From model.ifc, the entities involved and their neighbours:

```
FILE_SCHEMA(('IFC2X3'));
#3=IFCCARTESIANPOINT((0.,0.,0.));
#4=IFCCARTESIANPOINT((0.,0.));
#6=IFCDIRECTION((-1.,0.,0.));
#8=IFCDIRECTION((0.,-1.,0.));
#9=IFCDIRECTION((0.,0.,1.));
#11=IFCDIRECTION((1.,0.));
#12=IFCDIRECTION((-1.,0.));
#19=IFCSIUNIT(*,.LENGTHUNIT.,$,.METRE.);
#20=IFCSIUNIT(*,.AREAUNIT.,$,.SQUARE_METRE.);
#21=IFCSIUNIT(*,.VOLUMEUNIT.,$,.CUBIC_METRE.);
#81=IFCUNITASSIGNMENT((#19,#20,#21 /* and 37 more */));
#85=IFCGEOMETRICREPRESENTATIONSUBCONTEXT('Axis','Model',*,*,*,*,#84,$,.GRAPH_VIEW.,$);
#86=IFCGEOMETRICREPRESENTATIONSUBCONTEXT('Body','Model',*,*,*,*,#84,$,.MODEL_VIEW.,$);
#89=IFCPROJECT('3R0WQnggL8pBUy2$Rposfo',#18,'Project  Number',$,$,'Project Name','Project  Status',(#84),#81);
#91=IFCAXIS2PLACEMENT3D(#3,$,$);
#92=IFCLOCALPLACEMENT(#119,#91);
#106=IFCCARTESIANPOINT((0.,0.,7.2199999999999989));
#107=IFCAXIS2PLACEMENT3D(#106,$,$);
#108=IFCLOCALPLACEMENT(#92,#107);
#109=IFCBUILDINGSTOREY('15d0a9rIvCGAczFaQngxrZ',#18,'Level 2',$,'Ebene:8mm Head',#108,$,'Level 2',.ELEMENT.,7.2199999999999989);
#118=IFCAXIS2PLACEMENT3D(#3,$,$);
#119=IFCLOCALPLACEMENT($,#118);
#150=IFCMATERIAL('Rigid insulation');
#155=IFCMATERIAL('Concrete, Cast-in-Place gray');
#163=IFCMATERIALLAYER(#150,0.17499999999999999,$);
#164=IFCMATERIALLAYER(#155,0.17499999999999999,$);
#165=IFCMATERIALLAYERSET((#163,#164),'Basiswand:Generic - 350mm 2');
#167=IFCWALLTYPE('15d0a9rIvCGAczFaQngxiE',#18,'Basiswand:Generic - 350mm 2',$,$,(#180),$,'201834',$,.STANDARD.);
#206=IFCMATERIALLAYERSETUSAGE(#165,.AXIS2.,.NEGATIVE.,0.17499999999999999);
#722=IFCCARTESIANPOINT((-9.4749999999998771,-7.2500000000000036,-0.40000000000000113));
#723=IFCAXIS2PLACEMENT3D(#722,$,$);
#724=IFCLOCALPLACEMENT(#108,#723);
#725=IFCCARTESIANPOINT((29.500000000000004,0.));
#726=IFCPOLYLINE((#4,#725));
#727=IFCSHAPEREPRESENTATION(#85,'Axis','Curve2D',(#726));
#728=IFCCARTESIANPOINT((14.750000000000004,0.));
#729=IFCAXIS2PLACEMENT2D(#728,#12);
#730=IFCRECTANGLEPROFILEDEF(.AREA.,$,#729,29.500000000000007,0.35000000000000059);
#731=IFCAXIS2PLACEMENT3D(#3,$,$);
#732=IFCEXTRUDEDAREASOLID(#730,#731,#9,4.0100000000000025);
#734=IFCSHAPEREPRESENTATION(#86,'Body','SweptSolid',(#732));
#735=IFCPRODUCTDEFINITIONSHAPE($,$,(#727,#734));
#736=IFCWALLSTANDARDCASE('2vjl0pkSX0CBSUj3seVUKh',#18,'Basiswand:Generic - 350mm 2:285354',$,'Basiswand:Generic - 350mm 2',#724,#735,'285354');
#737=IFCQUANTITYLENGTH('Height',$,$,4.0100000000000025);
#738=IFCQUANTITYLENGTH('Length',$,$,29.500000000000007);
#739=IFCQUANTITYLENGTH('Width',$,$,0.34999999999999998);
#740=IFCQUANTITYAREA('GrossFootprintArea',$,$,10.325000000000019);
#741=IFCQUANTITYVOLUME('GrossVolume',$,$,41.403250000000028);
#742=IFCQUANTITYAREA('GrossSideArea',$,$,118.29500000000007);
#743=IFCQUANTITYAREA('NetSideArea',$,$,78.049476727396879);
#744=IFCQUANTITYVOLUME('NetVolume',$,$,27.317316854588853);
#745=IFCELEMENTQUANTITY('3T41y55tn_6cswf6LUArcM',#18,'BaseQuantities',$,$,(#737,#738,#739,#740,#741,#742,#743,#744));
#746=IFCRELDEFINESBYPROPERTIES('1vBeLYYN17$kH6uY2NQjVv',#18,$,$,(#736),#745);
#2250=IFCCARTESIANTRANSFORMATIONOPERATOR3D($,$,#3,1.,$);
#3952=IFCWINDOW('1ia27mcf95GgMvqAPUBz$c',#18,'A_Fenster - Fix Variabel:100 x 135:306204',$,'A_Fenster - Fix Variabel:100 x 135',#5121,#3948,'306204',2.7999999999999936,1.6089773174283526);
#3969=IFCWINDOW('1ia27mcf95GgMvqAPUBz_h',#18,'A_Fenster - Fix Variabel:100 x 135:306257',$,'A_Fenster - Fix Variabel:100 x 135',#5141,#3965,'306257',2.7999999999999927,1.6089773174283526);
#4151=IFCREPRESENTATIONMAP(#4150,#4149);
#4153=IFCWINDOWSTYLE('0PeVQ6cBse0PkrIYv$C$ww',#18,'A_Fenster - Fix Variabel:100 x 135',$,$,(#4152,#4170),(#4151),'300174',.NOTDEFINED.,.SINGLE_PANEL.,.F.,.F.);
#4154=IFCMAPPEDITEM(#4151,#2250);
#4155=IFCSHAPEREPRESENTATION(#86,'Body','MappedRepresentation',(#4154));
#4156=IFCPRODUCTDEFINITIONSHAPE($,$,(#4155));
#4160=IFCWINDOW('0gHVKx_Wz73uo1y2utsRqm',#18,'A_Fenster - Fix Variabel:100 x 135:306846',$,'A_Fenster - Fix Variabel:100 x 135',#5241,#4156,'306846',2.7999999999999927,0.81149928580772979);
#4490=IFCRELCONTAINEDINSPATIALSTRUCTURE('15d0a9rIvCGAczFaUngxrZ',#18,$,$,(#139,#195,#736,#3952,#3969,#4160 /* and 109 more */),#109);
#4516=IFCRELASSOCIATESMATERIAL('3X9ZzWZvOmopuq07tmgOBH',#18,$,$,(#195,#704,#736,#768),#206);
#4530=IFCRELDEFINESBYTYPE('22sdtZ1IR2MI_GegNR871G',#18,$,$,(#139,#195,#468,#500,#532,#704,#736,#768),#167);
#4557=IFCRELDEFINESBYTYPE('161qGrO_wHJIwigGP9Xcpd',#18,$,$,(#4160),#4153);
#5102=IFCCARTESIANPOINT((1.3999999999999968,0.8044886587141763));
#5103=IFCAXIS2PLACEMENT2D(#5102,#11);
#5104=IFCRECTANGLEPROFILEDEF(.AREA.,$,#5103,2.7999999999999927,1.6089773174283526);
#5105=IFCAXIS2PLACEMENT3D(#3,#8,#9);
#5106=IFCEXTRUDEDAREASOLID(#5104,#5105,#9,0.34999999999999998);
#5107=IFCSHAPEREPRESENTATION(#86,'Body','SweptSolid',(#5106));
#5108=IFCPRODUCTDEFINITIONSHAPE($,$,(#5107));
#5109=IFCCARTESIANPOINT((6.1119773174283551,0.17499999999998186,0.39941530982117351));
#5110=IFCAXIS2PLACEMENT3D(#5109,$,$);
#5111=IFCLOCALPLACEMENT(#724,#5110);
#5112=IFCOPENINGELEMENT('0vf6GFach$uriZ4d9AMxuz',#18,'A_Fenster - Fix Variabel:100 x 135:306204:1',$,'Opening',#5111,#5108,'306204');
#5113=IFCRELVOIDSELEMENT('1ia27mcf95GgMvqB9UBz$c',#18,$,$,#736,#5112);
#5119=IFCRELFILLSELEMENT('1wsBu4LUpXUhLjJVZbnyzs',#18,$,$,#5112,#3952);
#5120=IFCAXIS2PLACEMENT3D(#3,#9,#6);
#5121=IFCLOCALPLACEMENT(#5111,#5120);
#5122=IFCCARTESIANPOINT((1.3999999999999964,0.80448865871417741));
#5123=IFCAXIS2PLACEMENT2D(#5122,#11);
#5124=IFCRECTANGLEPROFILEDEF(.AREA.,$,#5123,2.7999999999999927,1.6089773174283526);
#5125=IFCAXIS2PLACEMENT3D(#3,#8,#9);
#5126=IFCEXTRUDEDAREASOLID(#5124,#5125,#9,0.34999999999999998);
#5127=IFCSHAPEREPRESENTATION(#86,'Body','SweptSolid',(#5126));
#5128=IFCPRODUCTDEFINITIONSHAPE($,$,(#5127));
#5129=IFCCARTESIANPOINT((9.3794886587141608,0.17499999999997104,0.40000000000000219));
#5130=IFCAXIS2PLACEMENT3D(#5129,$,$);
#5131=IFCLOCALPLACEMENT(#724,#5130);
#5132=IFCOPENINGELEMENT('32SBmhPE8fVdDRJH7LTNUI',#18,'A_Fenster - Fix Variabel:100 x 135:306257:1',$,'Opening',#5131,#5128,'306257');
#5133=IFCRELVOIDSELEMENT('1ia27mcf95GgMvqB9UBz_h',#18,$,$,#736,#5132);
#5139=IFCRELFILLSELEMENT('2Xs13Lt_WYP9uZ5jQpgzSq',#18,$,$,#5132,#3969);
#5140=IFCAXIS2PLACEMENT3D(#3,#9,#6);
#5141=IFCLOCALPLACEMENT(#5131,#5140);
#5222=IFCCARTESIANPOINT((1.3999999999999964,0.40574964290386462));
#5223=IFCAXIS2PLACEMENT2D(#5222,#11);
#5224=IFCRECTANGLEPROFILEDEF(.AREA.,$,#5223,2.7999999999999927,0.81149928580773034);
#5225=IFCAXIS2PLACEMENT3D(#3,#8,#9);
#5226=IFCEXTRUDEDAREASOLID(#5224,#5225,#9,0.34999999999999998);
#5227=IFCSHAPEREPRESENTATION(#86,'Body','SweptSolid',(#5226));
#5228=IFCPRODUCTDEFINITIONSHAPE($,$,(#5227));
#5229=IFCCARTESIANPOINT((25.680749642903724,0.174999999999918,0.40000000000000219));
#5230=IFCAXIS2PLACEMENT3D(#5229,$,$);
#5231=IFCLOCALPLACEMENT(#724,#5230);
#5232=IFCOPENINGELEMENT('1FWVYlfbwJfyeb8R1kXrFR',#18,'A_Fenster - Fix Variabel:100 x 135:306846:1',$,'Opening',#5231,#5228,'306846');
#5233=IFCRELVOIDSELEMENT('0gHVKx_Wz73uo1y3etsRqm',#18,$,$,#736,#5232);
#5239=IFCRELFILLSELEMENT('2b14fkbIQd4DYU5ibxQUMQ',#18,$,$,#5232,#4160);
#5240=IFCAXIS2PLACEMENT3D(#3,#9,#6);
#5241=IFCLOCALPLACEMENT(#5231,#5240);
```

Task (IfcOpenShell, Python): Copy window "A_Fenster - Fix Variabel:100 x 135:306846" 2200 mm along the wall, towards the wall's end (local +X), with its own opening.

```python
import ifcopenshell
import ifcopenshell.api.feature
import ifcopenshell.api.geometry
import ifcopenshell.api.pset
import ifcopenshell.api.root
import ifcopenshell.geom
import ifcopenshell.util.element
import ifcopenshell.util.placement
import ifcopenshell.util.shape
import ifcopenshell.util.unit

model = ifcopenshell.open("model.ifc")
unit_scale = ifcopenshell.util.unit.calculate_unit_scale(model)
area_scale = ifcopenshell.util.unit.calculate_unit_scale(model, "AREAUNIT")
volume_scale = ifcopenshell.util.unit.calculate_unit_scale(model, "VOLUMEUNIT")
settings = ifcopenshell.geom.settings()


def volume(element):
    """Net volume in cubic metres, openings subtracted."""
    shape = ifcopenshell.geom.create_shape(settings, element)
    return ifcopenshell.util.shape.get_volume(shape.geometry)


def reuse_history(source, copy):
    """copy_class also copies each property set's owner history, people and application; keep the originals."""
    for rel in copy.IsDefinedBy:
        if rel.is_a("IfcRelDefinesByProperties") and (history := rel.RelatingPropertyDefinition.OwnerHistory):
            rel.RelatingPropertyDefinition.OwnerHistory = source.OwnerHistory
            ifcopenshell.util.element.remove_deep2(model, history)


window = model.by_guid("0gHVKx_Wz73uo1y2utsRqm")
opening = window.FillsVoids[0].RelatingOpeningElement
wall = opening.VoidsElements[0].RelatingBuildingElement
before = volume(wall)
shift = ifcopenshell.util.placement.get_local_placement(wall.ObjectPlacement)[:3, 0] * 2.2 / unit_scale

# copy_class copies the void relationship, type, container and properties, but no geometry.
new_opening = ifcopenshell.api.root.copy_class(model, product=opening)
new_opening.Representation = ifcopenshell.util.element.copy_deep(
    model, opening.Representation, exclude=["IfcGeometricRepresentationContext", "IfcRepresentationMap"]
)
new_opening.Name = "A_Fenster - Fix Variabel:100 x 135"
new_opening.Tag = None
reuse_history(opening, new_opening)
new_window = ifcopenshell.api.root.copy_class(model, product=window)
new_window.Representation = ifcopenshell.util.element.copy_deep(
    model, window.Representation, exclude=["IfcGeometricRepresentationContext", "IfcRepresentationMap"]
)
new_window.Name = "A_Fenster - Fix Variabel:100 x 135"
new_window.Tag = None
reuse_history(window, new_window)
fills = ifcopenshell.api.feature.add_filling(model, opening=new_opening, element=new_window)
fills.OwnerHistory = new_window.OwnerHistory  # required in IFC2X3

for old, new in ((opening, new_opening), (window, new_window)):
    matrix = ifcopenshell.util.placement.get_local_placement(old.ObjectPlacement)
    matrix[:3, 3] += shift
    ifcopenshell.api.geometry.edit_object_placement(model, product=new, matrix=matrix, is_si=False)

after = volume(wall)
thickness = 0.35  # wall thickness in metres

# Update the wall's stored quantities.
qto = model.by_id(ifcopenshell.util.element.get_pset(wall, "BaseQuantities", should_inherit=False)["id"])
ifcopenshell.api.pset.edit_qto(model, qto=qto, properties={
    "NetSideArea": after / thickness / area_scale,
    "NetVolume": after / volume_scale,
})

print(f"wall volume {before:.3f} -> {after:.3f} m3")

model.write("model_edited.ifc")
```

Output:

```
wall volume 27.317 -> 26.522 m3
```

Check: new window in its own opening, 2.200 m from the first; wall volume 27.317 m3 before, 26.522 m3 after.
